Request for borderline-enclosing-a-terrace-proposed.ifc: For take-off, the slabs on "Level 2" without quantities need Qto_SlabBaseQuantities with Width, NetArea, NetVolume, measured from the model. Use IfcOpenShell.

First a look at what the model holds.

```python
import ifcopenshell
import ifcopenshell.util.element
import ifcopenshell.util.unit

model = ifcopenshell.open("borderline-enclosing-a-terrace-proposed.ifc")
print(model.schema)
for unit_type in ("LENGTHUNIT", "AREAUNIT", "VOLUMEUNIT"):
    print(unit_type, ifcopenshell.util.unit.calculate_unit_scale(model, unit_type))
storey = next(s for s in model.by_type("IfcBuildingStorey") if s.Name == "Level 2")
slabs = [e for e in ifcopenshell.util.element.get_decomposition(storey) if e.is_a("IfcSlab")]
for e in sorted(slabs, key=lambda e: e.id()):
    print(e.id(), e.is_a(), e.Name, list(ifcopenshell.util.element.get_psets(e, qtos_only=True)), sep=" | ")
```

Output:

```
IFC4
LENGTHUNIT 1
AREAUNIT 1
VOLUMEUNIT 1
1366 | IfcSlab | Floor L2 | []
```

```python
import ifcopenshell
import ifcopenshell.api.pset
import ifcopenshell.geom
import ifcopenshell.util.element
import ifcopenshell.util.shape
import ifcopenshell.util.unit

model = ifcopenshell.open("borderline-enclosing-a-terrace-proposed.ifc")
unit_scale = ifcopenshell.util.unit.calculate_unit_scale(model)
area_scale = ifcopenshell.util.unit.calculate_unit_scale(model, "AREAUNIT")
volume_scale = ifcopenshell.util.unit.calculate_unit_scale(model, "VOLUMEUNIT")
settings = ifcopenshell.geom.settings()

storey = next(s for s in model.by_type("IfcBuildingStorey") if s.Name == "Level 2")
slabs = [e for e in ifcopenshell.util.element.get_decomposition(storey) if e.is_a("IfcSlab")]

for e in sorted(slabs, key=lambda e: e.id()):
    if ifcopenshell.util.element.get_psets(e, qtos_only=True, should_inherit=False):
        continue
    # Geometry comes back in metres, in the element's own axes.
    shape = ifcopenshell.geom.create_shape(settings, e)
    values = {
        "Width": ifcopenshell.util.shape.get_z(shape.geometry) / unit_scale,
        "NetArea": ifcopenshell.util.shape.get_footprint_area(shape.geometry) / area_scale,
        "NetVolume": ifcopenshell.util.shape.get_volume(shape.geometry) / volume_scale,
    }
    qto = ifcopenshell.api.pset.add_qto(model, product=e, name="Qto_SlabBaseQuantities")
    ifcopenshell.api.pset.edit_qto(model, qto=qto, properties=values)
    print(e.id(), {k: round(v, 3) for k, v in values.items()})

model.write("borderline-enclosing-a-terrace-proposed_rev.ifc")
```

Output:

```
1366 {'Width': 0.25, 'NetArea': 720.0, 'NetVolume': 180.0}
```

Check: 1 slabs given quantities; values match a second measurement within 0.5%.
